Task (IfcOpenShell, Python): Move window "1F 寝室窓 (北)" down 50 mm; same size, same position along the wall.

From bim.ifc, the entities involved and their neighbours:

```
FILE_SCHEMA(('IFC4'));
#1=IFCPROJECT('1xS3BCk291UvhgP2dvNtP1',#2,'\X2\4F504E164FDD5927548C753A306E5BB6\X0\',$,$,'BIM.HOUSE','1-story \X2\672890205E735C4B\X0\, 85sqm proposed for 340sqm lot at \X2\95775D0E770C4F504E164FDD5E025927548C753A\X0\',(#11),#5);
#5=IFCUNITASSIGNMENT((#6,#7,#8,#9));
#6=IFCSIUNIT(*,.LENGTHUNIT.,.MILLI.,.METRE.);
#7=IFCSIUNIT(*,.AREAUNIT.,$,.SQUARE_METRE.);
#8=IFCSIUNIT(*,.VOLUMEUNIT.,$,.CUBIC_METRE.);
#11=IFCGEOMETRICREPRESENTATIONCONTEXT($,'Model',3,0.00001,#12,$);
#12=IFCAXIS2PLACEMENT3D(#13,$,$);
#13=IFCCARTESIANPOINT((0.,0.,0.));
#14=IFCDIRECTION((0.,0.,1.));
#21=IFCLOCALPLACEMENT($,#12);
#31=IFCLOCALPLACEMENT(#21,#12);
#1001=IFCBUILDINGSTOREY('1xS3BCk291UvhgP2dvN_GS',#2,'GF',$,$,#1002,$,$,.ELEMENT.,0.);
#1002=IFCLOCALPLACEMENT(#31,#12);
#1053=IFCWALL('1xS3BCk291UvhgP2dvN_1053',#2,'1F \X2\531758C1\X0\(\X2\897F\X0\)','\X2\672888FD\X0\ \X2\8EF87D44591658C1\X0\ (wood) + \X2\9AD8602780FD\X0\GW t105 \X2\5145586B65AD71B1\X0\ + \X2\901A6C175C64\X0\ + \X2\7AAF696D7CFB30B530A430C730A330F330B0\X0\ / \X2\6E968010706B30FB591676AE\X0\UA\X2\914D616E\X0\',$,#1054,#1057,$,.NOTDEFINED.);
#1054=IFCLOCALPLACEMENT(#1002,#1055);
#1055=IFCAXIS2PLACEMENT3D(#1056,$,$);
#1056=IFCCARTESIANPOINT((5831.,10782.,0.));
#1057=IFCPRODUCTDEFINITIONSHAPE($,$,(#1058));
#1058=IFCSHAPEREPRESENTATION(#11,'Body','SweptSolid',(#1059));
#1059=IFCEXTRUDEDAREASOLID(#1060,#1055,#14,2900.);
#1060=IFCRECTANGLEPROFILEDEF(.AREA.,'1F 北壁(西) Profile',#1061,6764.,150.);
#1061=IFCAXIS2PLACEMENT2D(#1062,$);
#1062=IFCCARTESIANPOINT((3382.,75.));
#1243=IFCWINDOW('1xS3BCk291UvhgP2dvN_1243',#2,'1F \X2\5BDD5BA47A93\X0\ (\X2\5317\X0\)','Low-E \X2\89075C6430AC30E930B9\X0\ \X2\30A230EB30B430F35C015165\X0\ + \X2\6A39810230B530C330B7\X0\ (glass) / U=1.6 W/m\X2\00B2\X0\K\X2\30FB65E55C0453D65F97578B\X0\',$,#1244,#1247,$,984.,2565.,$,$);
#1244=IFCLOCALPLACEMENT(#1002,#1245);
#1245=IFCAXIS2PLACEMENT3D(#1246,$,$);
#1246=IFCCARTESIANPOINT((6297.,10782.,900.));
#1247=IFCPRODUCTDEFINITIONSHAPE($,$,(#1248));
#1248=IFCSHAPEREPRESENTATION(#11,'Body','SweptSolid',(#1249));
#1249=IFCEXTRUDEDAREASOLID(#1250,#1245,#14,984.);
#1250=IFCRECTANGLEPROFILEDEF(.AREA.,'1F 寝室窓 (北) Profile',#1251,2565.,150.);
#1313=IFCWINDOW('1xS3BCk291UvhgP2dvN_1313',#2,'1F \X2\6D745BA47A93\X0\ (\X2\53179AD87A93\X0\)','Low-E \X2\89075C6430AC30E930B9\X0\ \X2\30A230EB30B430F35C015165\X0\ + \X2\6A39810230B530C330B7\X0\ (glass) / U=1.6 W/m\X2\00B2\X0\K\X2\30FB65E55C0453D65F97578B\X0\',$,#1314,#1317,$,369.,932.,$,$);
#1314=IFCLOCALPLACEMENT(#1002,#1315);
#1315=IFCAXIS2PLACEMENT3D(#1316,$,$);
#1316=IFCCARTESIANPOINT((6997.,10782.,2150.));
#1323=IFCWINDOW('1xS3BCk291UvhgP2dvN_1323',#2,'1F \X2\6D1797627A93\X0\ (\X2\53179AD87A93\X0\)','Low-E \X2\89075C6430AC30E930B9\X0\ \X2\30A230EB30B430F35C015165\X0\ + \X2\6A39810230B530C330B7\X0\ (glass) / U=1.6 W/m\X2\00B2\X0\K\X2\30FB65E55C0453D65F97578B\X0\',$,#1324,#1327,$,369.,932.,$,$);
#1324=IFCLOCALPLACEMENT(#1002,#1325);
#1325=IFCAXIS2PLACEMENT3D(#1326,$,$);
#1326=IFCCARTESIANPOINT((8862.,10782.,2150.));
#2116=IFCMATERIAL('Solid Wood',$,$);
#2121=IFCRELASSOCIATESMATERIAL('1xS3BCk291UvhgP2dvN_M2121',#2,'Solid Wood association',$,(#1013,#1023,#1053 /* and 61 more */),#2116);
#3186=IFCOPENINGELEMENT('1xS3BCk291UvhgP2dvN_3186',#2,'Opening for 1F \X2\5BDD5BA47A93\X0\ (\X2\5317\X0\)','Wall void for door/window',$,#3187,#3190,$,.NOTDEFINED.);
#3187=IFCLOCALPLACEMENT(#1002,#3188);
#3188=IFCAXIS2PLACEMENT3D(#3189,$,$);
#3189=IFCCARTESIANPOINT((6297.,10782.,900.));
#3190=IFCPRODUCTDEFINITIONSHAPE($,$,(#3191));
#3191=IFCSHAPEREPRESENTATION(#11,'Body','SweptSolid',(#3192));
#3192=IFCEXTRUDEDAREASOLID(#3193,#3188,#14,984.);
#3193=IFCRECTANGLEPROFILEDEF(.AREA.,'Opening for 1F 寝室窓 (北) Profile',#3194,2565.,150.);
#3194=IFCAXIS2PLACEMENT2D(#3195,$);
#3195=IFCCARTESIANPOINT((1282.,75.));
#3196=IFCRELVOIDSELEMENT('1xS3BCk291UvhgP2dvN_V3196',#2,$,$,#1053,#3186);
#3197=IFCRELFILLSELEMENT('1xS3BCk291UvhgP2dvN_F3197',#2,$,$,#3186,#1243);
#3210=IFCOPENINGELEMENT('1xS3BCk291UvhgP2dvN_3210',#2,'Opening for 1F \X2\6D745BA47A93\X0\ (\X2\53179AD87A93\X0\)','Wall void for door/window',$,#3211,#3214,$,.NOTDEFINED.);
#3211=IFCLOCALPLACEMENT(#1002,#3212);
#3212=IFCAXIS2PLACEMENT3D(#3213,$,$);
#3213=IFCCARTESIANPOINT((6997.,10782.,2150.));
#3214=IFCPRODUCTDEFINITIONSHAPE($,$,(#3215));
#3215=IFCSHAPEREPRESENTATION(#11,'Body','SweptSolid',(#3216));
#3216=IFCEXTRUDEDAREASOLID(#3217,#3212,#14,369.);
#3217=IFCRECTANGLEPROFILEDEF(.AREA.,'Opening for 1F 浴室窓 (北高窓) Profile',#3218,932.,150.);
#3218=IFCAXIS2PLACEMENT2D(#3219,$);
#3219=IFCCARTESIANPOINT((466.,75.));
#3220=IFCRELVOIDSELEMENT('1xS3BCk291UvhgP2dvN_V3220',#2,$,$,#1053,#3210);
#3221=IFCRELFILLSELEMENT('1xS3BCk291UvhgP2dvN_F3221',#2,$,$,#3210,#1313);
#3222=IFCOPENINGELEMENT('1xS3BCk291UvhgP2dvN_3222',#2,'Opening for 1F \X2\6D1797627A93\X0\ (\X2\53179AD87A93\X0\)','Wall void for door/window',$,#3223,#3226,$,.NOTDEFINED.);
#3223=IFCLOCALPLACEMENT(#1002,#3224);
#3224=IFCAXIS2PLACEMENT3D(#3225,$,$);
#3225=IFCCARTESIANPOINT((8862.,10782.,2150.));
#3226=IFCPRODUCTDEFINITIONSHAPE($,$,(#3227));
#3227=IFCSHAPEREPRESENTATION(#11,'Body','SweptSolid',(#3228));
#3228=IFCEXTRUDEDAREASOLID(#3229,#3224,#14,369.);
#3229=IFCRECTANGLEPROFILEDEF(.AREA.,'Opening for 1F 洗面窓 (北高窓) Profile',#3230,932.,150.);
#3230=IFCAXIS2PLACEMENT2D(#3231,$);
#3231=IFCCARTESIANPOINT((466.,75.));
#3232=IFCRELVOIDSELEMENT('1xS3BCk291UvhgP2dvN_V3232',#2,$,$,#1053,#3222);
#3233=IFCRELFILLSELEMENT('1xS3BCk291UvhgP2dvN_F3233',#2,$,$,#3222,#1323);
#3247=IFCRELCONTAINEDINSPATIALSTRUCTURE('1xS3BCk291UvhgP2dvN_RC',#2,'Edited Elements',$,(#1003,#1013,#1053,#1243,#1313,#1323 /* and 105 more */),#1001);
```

```python
import numpy as np
import ifcopenshell
import ifcopenshell.api.geometry
import ifcopenshell.util.placement
import ifcopenshell.util.unit

model = ifcopenshell.open("bim.ifc")
unit_scale = ifcopenshell.util.unit.calculate_unit_scale(model)

window = model.by_guid("1xS3BCk291UvhgP2dvN_1243")
opening = window.FillsVoids[0].RelatingOpeningElement
dz = -0.05 / unit_scale

shift = np.array([0.0, 0.0, dz])
# The window is not placed relative to its opening, so move both.
for product in (opening, window):
    matrix = ifcopenshell.util.placement.get_local_placement(product.ObjectPlacement)
    matrix[:3, 3] += shift
    ifcopenshell.api.geometry.edit_object_placement(model, product=product, matrix=matrix, is_si=False)

print(f"moved by {dz * unit_scale:+.3f} m")

model.write("bim_rev.ifc")
```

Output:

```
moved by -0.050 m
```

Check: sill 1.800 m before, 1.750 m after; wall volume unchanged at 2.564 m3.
